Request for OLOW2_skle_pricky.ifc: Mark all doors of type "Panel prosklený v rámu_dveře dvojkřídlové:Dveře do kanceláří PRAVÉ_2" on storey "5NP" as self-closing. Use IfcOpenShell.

First a look at what the model holds.

```python
import ifcopenshell
import ifcopenshell.util.element

model = ifcopenshell.open("OLOW2_skle_pricky.ifc")
print(model.schema)
storey = next(s for s in model.by_type("IfcBuildingStorey") if s.Name == "5NP")
doors = [e for e in ifcopenshell.util.element.get_decomposition(storey) if e.is_a("IfcDoor")]
seen = {}
for e in doors:
    element_type = ifcopenshell.util.element.get_type(e)
    key = (element_type.Name if element_type != e and element_type else None, ifcopenshell.util.element.get_pset(e, "Pset_DoorCommon", "SelfClosing"))
    seen[key] = seen.get(key, 0) + 1
for (name, value), count in sorted(seen.items(), key=str):
    print(count, "x", name, "|", value)
```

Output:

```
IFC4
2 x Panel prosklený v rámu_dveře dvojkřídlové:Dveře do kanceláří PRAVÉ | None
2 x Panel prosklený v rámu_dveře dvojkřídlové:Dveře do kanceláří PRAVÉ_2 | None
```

```python
import ifcopenshell
import ifcopenshell.api.pset
import ifcopenshell.util.element

model = ifcopenshell.open("OLOW2_skle_pricky.ifc")

storey = next(s for s in model.by_type("IfcBuildingStorey") if s.Name == "5NP")
doors = [e for e in ifcopenshell.util.element.get_decomposition(storey) if e.is_a("IfcDoor")]

count = 0
for e in doors:
    element_type = ifcopenshell.util.element.get_type(e)
    if element_type in (None, e) or element_type.Name != "Panel prosklený v rámu_dveře dvojkřídlové:Dveře do kanceláří PRAVÉ_2":
        continue
    # add_pset returns the element's existing set when there is one.
    pset = ifcopenshell.api.pset.add_pset(model, product=e, name="Pset_DoorCommon")
    ifcopenshell.api.pset.edit_pset(model, pset=pset, properties={"SelfClosing": True})
    count += 1

print(count, "doors updated")

model.write("OLOW2_skle_pricky_updated.ifc")
```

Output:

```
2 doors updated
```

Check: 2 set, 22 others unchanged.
